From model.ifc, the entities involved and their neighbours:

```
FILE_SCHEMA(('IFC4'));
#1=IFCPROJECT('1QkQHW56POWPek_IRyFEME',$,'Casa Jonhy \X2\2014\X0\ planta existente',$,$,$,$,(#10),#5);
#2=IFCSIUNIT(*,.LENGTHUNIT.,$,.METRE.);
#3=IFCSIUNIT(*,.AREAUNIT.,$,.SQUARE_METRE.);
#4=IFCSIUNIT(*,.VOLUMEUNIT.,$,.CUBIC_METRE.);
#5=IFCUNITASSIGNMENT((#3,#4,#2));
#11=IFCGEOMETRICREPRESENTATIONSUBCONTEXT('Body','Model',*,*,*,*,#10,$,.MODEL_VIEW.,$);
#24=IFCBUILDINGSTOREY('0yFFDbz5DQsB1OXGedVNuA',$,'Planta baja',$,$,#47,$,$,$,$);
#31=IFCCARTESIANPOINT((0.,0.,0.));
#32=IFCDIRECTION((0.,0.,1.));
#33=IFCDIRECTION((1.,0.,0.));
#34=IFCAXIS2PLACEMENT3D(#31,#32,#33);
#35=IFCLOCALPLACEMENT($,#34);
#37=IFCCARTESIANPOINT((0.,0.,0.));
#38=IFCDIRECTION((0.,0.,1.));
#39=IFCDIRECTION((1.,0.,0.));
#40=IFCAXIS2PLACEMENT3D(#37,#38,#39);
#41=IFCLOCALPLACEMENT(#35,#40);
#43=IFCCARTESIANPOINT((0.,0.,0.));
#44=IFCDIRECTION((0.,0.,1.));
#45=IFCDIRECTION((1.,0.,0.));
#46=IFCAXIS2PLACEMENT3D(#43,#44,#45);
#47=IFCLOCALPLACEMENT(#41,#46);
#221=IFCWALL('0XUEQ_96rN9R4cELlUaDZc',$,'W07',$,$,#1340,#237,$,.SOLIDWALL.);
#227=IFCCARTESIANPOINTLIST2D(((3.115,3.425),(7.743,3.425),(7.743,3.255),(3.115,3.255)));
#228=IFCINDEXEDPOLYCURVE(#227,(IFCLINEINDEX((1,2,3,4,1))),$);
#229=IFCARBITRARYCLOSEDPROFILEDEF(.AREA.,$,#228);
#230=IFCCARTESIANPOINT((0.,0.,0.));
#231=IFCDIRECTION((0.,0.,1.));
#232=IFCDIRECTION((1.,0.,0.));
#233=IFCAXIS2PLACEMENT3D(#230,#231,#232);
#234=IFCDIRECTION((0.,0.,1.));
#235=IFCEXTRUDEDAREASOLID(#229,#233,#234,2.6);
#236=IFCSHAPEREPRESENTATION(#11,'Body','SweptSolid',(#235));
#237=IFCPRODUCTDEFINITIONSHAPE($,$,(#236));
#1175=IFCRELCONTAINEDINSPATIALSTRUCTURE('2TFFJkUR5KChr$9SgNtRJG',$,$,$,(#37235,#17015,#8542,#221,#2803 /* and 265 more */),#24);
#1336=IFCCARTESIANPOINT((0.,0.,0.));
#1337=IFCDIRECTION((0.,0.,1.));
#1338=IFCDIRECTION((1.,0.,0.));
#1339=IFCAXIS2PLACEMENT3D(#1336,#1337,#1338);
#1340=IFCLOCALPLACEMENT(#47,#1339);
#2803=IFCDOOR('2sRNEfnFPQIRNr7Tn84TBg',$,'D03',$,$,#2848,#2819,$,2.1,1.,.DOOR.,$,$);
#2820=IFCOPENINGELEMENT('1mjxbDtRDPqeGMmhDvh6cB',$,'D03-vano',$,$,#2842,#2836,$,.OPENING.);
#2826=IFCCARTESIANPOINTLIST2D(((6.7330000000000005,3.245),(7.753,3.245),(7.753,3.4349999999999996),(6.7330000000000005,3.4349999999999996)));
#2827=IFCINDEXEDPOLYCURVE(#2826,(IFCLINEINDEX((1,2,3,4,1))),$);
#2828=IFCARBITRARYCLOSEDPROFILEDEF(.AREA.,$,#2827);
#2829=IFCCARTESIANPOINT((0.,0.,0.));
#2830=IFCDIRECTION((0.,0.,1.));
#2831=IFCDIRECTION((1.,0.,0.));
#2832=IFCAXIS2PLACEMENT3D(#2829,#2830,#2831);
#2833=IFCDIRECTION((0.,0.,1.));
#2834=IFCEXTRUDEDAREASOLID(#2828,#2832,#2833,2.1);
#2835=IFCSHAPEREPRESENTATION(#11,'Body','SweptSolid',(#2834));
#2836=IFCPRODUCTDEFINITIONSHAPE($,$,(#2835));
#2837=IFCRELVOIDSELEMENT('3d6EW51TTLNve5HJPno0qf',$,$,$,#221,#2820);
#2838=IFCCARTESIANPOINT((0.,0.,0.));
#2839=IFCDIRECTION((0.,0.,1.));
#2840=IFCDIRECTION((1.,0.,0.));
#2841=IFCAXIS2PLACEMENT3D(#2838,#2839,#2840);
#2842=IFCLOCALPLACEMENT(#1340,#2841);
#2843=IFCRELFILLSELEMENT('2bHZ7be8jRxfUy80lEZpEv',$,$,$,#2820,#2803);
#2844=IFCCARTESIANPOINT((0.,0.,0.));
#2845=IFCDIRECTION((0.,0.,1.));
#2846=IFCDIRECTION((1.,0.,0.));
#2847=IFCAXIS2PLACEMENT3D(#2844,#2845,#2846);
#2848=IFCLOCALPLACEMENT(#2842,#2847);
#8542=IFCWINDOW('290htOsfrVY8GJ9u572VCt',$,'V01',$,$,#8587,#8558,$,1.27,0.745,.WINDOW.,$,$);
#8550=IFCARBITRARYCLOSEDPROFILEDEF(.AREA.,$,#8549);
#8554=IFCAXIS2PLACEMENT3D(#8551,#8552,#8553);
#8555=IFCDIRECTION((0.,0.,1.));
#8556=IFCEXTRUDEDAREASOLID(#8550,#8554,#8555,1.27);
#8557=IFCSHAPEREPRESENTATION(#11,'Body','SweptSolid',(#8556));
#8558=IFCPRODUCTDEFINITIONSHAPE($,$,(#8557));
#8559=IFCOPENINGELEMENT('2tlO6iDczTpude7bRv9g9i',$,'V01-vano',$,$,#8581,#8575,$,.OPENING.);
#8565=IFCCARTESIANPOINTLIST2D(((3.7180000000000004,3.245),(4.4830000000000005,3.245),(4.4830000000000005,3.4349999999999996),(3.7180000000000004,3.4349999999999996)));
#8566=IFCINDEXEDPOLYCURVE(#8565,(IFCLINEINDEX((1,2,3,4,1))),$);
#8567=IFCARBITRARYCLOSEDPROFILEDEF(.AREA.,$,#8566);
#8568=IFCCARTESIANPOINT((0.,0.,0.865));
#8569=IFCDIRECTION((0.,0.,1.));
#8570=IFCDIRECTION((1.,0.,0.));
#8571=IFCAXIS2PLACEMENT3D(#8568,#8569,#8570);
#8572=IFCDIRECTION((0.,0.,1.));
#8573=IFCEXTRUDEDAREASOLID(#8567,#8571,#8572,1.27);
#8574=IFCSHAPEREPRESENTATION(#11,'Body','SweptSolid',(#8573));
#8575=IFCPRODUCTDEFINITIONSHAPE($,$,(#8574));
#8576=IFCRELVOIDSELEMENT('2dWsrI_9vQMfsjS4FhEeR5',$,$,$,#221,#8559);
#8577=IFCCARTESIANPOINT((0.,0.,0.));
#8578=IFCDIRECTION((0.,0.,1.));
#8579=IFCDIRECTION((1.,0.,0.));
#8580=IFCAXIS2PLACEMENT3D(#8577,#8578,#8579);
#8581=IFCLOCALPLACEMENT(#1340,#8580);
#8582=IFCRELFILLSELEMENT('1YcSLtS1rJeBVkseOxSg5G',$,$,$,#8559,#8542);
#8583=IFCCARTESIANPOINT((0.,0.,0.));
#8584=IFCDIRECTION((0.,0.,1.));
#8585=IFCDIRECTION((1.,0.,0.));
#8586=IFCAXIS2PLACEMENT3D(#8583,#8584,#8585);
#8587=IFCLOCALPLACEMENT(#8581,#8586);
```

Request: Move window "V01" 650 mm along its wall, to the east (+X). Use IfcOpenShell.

```python
import ifcopenshell
import ifcopenshell.api.geometry
import ifcopenshell.util.placement
import ifcopenshell.util.unit

model = ifcopenshell.open("model.ifc")
unit_scale = ifcopenshell.util.unit.calculate_unit_scale(model)

window = model.by_id(8542)
opening = window.FillsVoids[0].RelatingOpeningElement
wall = opening.VoidsElements[0].RelatingBuildingElement

wall_matrix = ifcopenshell.util.placement.get_local_placement(wall.ObjectPlacement)
shift = wall_matrix[:3, 0] * 0.65 / unit_scale
before = ifcopenshell.util.placement.get_local_placement(window.ObjectPlacement)[:3, 3].copy()

# The window is placed relative to its opening, so it follows when the opening moves.
matrix = ifcopenshell.util.placement.get_local_placement(opening.ObjectPlacement)
matrix[:3, 3] += shift
ifcopenshell.api.geometry.edit_object_placement(
    model, product=opening, matrix=matrix, is_si=False, should_transform_children=True
)

after = ifcopenshell.util.placement.get_local_placement(window.ObjectPlacement)[:3, 3]
print("window moved by", (after - before).round(3) + 0.0)

model.write("model_rev.ifc")
```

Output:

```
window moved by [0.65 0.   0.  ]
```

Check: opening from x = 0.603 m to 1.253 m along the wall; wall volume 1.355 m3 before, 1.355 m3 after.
